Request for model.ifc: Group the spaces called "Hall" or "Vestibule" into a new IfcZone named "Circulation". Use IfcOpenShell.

First a look at what the model holds.

```python
import ifcopenshell

model = ifcopenshell.open("model.ifc")
print(model.schema)
seen = {}
for space in model.by_type("IfcSpace"):
    seen[space.LongName] = seen.get(space.LongName, 0) + 1
for name, count in sorted(seen.items(), key=str):
    print(count, "x", name)
print("zones:", [z.Name for z in model.by_type("IfcZone")][:20])
```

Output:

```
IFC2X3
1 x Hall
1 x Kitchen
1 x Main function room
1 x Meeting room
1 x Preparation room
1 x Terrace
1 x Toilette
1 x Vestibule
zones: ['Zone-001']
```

```python
import ifcopenshell
import ifcopenshell.api.group
import ifcopenshell.api.root

model = ifcopenshell.open("model.ifc")

names = {"Hall", "Vestibule"}
spaces = [s for s in model.by_type("IfcSpace") if s.LongName in names]

zone = ifcopenshell.api.root.create_entity(model, ifc_class="IfcZone", name="Circulation")
ifcopenshell.api.group.assign_group(model, products=spaces, group=zone)
print(len(spaces), "spaces in", zone.Name)

model.write("model_rev.ifc")
```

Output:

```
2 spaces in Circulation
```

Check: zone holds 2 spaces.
